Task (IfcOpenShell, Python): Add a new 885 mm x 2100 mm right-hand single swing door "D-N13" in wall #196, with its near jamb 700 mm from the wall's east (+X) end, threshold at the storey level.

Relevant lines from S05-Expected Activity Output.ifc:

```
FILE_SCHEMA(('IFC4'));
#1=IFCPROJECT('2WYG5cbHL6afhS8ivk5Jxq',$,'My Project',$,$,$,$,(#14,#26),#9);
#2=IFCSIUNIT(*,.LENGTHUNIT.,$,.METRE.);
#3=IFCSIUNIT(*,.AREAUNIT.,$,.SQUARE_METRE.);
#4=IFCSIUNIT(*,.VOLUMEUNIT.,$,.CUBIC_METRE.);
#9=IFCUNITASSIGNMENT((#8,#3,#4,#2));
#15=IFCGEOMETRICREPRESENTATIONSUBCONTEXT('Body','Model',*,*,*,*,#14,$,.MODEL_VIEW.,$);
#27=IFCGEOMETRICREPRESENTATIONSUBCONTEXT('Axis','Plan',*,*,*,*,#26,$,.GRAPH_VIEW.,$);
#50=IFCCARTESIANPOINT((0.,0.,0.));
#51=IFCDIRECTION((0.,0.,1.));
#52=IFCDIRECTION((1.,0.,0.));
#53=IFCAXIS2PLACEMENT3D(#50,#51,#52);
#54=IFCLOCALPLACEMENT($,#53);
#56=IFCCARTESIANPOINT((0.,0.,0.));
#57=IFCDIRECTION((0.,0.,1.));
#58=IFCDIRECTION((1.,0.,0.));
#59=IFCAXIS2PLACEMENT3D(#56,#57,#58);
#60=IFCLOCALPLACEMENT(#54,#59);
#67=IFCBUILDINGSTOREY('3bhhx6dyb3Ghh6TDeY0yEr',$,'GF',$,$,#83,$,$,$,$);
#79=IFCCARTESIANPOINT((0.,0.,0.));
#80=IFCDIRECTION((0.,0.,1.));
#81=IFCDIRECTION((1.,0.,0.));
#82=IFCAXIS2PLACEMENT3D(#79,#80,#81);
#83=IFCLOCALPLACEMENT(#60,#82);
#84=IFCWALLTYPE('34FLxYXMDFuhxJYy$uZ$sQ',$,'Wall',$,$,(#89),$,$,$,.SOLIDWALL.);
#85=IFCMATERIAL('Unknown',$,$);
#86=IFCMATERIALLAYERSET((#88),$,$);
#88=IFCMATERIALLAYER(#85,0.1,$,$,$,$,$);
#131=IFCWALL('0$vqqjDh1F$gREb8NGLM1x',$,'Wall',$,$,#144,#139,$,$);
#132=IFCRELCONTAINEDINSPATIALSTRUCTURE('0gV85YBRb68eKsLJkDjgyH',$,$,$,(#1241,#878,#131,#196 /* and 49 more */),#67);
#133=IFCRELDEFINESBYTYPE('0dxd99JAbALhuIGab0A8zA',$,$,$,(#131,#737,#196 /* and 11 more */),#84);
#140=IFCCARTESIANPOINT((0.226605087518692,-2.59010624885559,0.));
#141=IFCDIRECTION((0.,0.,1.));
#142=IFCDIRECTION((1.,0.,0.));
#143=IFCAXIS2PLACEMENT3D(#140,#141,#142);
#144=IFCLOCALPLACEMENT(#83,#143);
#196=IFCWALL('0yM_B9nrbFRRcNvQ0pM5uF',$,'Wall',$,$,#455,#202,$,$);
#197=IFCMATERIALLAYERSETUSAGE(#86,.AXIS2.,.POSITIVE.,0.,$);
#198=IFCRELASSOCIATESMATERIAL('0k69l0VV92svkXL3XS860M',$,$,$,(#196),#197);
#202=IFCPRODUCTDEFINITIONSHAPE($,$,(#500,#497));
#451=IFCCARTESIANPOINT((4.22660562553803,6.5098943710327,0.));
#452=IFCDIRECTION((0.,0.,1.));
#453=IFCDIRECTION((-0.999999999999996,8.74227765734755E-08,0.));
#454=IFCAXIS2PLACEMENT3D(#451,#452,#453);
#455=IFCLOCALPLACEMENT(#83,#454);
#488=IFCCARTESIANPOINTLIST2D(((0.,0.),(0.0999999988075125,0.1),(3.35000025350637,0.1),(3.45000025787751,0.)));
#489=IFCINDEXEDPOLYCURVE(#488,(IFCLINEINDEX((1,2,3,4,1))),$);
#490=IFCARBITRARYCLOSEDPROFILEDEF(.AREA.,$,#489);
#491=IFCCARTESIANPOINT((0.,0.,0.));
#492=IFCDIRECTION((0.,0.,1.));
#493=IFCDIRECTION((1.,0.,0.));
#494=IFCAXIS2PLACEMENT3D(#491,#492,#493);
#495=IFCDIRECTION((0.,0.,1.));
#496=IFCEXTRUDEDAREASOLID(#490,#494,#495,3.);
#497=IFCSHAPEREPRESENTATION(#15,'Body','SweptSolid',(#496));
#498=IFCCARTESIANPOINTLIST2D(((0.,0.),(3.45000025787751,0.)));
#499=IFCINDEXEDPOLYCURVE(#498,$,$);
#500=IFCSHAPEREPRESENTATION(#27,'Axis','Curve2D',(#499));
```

```python
import numpy as np
import ifcopenshell
import ifcopenshell.api.feature
import ifcopenshell.api.geometry
import ifcopenshell.api.root
import ifcopenshell.api.spatial
import ifcopenshell.geom
import ifcopenshell.util.element
import ifcopenshell.util.placement
import ifcopenshell.util.representation
import ifcopenshell.util.shape
import ifcopenshell.util.unit

model = ifcopenshell.open("S05-Expected Activity Output.ifc")
unit_scale = ifcopenshell.util.unit.calculate_unit_scale(model)
settings = ifcopenshell.geom.settings()


def volume(element):
    """Net volume in cubic metres, openings subtracted."""
    shape = ifcopenshell.geom.create_shape(settings, element)
    return ifcopenshell.util.shape.get_volume(shape.geometry)


wall = model.by_guid("0yM_B9nrbFRRcNvQ0pM5uF")
storey = ifcopenshell.util.element.get_container(wall, ifc_class="IfcBuildingStorey")
context = ifcopenshell.util.representation.get_context(model, "Model", "Body", "MODEL_VIEW")
before = volume(wall)

width, height, from_end, sill = 0.885, 2.1, 0.7, 0.0  # metres

# The wall runs along its own X axis, and the end named is its -X end.
wall_shape = ifcopenshell.geom.create_shape(settings, wall)
x, y, z = ifcopenshell.util.shape.get_vertices(wall_shape.geometry).T
start = x.min() + from_end
face, thickness = float(y.min()), float(y.max() - y.min())
wall_matrix = ifcopenshell.util.placement.get_local_placement(wall.ObjectPlacement)
level = ifcopenshell.util.placement.get_local_placement(storey.ObjectPlacement)[2, 3]


def in_wall(x, y):
    """Placement at x, y metres in the wall's axes, at sill height."""
    matrix = wall_matrix.copy()
    matrix[:, 3] = wall_matrix @ np.array([x / unit_scale, y / unit_scale, 0.0, 1.0])
    matrix[2, 3] = level + sill / unit_scale
    return matrix


# Opening: a box that overshoots both wall faces by 50 mm.
opening = ifcopenshell.api.root.create_entity(model, ifc_class="IfcOpeningElement", predefined_type="OPENING")
box = ifcopenshell.api.geometry.add_wall_representation(
    model, context=context, length=width, height=height, thickness=thickness + 0.1
)
ifcopenshell.api.geometry.assign_representation(model, product=opening, representation=box)
ifcopenshell.api.geometry.edit_object_placement(model, product=opening, matrix=in_wall(start, face - 0.05), is_si=False)
ifcopenshell.api.feature.add_feature(model, feature=opening, element=wall)

door = ifcopenshell.api.root.create_entity(model, ifc_class="IfcDoor", name="D-N13", predefined_type="DOOR")
door.OverallWidth, door.OverallHeight = width / unit_scale, height / unit_scale
door.OperationType = "SINGLE_SWING_RIGHT"
body = ifcopenshell.api.geometry.add_door_representation(
    model,
    context=context,
    overall_width=door.OverallWidth,
    overall_height=door.OverallHeight,
    operation_type="SINGLE_SWING_RIGHT",
    lining_properties={"LiningDepth": thickness / unit_scale, "ThresholdDepth": thickness / unit_scale},
)
ifcopenshell.api.geometry.assign_representation(model, product=door, representation=body)
ifcopenshell.api.spatial.assign_container(model, products=[door], relating_structure=storey)
ifcopenshell.api.feature.add_filling(model, opening=opening, element=door)

# The lining spans the wall, so the door starts at the wall face.
ifcopenshell.api.geometry.edit_object_placement(model, product=door, matrix=in_wall(start, face), is_si=False)

after = volume(wall)

print(f"wall volume {before:.3f} -> {after:.3f} m3")

model.write("S05-Expected Activity Output_updated.ifc")
```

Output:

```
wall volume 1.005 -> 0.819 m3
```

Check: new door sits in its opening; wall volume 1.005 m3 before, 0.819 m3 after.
